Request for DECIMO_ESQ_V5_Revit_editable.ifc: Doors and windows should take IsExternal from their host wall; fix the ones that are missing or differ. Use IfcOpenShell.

First a look at what the model holds.

```python
import ifcopenshell
import ifcopenshell.util.element

model = ifcopenshell.open("DECIMO_ESQ_V5_Revit_editable.ifc")
print(model.schema)
seen = {}
for e in model.by_type("IfcDoor") + model.by_type("IfcWindow"):
    if not e.FillsVoids:
        continue
    host = e.FillsVoids[0].RelatingOpeningElement.VoidsElements[0].RelatingBuildingElement
    own = ifcopenshell.util.element.get_pset(e, f"Pset_{e.is_a()[3:].removesuffix('StandardCase')}Common", "IsExternal")
    wall = ifcopenshell.util.element.get_pset(host, "Pset_WallCommon", "IsExternal")
    seen[e.is_a(), own, wall] = seen.get((e.is_a(), own, wall), 0) + 1
for (cls, own, wall), count in sorted(seen.items(), key=str):
    print(count, cls, "IsExternal:", own, "| host wall:", wall)
```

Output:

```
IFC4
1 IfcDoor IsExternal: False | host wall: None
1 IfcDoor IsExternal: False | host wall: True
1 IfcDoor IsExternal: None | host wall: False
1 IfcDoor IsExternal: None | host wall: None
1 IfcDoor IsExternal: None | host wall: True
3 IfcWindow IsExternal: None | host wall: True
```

```python
import ifcopenshell
import ifcopenshell.api.pset
import ifcopenshell.util.element

model = ifcopenshell.open("DECIMO_ESQ_V5_Revit_editable.ifc")

count = 0
for ifc_class, pset_name in (("IfcDoor", "Pset_DoorCommon"), ("IfcWindow", "Pset_WindowCommon")):
    for e in model.by_type(ifc_class):
        if not e.FillsVoids:
            continue
        host = e.FillsVoids[0].RelatingOpeningElement.VoidsElements[0].RelatingBuildingElement
        external = ifcopenshell.util.element.get_pset(host, "Pset_WallCommon", "IsExternal")
        if external is None or ifcopenshell.util.element.get_pset(e, pset_name, "IsExternal") == external:
            continue
        pset = ifcopenshell.api.pset.add_pset(model, product=e, name=pset_name)
        ifcopenshell.api.pset.edit_pset(model, pset=pset, properties={"IsExternal": external})
        count += 1

print(count, "updated")

model.write("DECIMO_ESQ_V5_Revit_editable-out.ifc")
```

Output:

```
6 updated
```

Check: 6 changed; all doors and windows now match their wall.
